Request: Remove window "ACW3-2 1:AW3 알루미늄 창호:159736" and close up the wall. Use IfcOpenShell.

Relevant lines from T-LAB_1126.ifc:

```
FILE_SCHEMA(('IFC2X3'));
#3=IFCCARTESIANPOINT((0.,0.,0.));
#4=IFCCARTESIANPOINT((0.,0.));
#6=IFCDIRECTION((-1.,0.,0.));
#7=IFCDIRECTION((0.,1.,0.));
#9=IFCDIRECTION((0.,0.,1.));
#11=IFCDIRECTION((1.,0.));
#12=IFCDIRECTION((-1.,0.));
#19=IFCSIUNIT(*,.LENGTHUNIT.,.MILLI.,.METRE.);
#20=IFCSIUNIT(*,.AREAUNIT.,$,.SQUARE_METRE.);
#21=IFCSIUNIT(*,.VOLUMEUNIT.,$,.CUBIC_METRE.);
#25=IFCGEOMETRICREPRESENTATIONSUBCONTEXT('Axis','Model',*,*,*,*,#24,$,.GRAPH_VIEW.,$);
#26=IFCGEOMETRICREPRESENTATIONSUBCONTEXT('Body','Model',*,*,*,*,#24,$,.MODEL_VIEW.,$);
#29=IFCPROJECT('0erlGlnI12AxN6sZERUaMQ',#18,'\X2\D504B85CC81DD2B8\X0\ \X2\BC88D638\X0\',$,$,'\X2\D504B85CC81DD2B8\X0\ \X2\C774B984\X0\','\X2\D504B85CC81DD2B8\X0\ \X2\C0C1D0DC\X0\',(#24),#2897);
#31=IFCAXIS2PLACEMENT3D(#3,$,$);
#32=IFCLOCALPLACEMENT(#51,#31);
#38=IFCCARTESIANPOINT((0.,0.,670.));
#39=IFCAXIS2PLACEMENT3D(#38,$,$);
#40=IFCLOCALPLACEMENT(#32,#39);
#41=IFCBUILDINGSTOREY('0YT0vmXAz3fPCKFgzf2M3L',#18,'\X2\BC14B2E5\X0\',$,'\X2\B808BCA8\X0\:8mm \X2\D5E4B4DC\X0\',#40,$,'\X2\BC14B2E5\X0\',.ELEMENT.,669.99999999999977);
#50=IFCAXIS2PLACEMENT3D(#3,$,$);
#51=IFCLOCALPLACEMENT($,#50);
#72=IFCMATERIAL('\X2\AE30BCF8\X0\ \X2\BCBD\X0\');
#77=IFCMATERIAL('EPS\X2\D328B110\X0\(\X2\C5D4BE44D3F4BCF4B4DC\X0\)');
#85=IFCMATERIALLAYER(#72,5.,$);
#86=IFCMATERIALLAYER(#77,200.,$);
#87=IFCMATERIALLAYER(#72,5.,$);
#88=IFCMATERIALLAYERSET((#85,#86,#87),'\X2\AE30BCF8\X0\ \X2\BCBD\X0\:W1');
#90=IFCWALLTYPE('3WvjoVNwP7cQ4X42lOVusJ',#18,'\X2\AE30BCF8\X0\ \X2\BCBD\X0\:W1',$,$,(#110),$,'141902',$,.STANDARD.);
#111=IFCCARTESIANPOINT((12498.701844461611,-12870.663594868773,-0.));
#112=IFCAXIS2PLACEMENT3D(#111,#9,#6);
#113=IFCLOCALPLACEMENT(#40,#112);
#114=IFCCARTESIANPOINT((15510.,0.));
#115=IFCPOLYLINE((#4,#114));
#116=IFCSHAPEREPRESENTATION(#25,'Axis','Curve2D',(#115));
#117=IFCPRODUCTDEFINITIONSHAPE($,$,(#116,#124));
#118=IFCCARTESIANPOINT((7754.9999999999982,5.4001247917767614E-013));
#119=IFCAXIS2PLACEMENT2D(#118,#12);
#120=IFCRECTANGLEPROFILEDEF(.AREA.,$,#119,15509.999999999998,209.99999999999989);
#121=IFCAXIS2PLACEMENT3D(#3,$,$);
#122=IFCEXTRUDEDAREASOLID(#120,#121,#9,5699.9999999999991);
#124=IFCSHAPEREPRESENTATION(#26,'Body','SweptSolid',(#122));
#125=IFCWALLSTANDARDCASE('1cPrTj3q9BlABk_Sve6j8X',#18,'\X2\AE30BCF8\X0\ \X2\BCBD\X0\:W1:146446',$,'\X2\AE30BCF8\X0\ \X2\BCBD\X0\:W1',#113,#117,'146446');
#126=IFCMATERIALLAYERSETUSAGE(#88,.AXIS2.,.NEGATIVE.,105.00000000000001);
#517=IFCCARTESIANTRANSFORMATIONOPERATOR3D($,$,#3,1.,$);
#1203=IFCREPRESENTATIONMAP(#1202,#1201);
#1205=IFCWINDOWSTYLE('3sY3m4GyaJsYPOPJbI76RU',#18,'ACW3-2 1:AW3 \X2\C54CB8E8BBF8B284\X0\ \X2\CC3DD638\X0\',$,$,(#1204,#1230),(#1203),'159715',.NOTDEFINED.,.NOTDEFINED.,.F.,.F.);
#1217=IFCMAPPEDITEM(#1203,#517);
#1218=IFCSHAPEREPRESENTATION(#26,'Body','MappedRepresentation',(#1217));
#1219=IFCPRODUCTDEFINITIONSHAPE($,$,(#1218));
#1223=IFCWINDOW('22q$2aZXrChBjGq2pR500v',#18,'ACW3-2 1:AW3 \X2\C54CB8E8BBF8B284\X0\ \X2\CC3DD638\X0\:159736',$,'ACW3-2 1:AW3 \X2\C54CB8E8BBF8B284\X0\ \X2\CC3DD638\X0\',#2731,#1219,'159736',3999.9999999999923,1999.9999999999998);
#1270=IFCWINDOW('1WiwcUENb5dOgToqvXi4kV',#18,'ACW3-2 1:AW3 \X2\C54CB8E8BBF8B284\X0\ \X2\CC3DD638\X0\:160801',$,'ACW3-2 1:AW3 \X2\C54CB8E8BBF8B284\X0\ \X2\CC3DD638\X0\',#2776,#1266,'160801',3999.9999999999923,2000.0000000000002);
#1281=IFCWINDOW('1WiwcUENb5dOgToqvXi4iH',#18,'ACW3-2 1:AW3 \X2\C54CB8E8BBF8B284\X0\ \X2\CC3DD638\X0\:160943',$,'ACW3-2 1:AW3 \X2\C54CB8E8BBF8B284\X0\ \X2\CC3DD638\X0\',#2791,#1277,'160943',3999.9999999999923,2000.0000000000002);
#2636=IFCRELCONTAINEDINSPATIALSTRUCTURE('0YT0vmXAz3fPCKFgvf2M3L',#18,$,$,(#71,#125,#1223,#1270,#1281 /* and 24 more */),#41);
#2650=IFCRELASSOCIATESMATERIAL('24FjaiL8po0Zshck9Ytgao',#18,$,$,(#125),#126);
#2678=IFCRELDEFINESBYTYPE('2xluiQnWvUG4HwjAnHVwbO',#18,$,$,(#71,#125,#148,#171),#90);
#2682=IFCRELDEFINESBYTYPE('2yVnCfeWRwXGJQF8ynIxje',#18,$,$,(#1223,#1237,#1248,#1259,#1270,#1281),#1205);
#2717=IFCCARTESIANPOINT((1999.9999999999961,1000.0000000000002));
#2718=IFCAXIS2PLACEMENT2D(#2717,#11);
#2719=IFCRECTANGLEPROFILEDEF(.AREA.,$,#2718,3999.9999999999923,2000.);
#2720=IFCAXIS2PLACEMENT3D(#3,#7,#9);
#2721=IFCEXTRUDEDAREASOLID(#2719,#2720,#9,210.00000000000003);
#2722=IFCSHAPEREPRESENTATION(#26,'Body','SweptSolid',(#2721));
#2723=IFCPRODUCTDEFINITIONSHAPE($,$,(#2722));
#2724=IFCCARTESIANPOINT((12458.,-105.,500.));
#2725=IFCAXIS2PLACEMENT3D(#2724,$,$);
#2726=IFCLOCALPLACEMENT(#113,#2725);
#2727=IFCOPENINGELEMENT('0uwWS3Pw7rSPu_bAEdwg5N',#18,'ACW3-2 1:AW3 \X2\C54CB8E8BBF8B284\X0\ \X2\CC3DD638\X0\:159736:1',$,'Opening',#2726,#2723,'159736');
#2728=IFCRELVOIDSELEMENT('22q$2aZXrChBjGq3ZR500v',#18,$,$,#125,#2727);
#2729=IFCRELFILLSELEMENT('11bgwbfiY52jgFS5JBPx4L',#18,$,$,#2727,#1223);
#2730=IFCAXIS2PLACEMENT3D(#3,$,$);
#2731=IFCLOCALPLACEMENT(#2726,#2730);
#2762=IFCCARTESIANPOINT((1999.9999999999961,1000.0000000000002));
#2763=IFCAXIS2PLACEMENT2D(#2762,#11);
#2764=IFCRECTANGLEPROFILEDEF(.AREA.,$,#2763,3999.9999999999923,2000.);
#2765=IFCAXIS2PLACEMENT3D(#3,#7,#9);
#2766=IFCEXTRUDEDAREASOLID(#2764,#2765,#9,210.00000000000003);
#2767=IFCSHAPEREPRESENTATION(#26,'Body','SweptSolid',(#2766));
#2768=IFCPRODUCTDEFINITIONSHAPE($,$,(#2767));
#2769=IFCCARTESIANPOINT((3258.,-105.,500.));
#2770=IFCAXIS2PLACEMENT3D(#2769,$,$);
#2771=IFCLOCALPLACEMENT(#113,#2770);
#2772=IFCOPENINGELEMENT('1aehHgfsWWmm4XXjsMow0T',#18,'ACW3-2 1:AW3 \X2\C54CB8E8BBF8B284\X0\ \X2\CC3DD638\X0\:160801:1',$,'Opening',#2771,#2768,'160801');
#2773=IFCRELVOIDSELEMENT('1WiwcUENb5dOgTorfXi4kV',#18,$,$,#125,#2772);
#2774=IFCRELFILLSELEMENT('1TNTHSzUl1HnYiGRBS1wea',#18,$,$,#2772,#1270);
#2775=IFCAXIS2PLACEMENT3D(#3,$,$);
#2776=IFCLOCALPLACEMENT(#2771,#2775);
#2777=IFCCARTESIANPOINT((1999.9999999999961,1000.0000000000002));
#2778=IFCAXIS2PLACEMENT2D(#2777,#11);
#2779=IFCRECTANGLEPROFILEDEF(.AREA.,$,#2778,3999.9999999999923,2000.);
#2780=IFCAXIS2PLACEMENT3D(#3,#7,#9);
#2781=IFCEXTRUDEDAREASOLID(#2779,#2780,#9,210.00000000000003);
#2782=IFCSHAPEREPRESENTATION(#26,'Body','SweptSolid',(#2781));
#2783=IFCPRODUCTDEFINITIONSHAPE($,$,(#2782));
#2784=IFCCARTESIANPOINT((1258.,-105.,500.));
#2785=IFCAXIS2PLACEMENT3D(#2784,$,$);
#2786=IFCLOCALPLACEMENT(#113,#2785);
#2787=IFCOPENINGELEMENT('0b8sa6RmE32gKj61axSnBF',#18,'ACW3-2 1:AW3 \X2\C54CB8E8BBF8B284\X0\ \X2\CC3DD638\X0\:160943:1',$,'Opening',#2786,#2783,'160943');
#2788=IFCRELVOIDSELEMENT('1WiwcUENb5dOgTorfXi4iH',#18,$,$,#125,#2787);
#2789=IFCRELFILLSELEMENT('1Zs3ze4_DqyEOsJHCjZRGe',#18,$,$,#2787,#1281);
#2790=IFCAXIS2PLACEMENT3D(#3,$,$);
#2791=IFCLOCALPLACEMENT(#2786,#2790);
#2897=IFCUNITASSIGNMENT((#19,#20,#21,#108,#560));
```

```python
import ifcopenshell
import ifcopenshell.api.feature
import ifcopenshell.api.root
import ifcopenshell.geom
import ifcopenshell.util.shape

model = ifcopenshell.open("T-LAB_1126.ifc")
settings = ifcopenshell.geom.settings()


def volume(element):
    """Net volume in cubic metres, openings subtracted."""
    shape = ifcopenshell.geom.create_shape(settings, element)
    return ifcopenshell.util.shape.get_volume(shape.geometry)


window = model.by_guid("22q$2aZXrChBjGq2pR500v")
opening = window.FillsVoids[0].RelatingOpeningElement
wall = opening.VoidsElements[0].RelatingBuildingElement
before = volume(wall)

ifcopenshell.api.root.remove_product(model, product=window)
ifcopenshell.api.feature.remove_feature(model, feature=opening)

after = volume(wall)

print(f"wall volume {before:.3f} -> {after:.3f} m3")

model.write("T-LAB_1126_rev.ifc")
```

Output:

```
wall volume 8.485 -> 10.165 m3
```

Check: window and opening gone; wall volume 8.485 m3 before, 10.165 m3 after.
